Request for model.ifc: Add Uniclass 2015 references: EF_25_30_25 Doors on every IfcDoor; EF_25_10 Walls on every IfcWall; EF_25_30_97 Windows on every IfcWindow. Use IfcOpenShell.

First a look at what the model holds.

```python
import ifcopenshell

model = ifcopenshell.open("model.ifc")
print(model.schema)
print("classifications:", [c.Name for c in model.by_type("IfcClassification")])
for ifc_class in ("IfcDoor", "IfcRoof", "IfcStair", "IfcWall", "IfcWindow"):
    print(ifc_class, len(model.by_type(ifc_class)))
```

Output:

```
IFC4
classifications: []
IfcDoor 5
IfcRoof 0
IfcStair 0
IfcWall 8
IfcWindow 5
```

```python
import ifcopenshell
import ifcopenshell.api.classification

model = ifcopenshell.open("model.ifc")

system = ifcopenshell.api.classification.add_classification(model, classification="Uniclass 2015")

codes = {
    "IfcDoor": ("EF_25_30_25", "Doors"),
    "IfcWall": ("EF_25_10", "Walls"),
    "IfcWindow": ("EF_25_30_97", "Windows"),
}
for ifc_class, (code, name) in codes.items():
    products = model.by_type(ifc_class)
    ifcopenshell.api.classification.add_reference(
        model, products=products, classification=system, identification=code, name=name
    )
    print(code, len(products))

model.write("model_edited.ifc")
```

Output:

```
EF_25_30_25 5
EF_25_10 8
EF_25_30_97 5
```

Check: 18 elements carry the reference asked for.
